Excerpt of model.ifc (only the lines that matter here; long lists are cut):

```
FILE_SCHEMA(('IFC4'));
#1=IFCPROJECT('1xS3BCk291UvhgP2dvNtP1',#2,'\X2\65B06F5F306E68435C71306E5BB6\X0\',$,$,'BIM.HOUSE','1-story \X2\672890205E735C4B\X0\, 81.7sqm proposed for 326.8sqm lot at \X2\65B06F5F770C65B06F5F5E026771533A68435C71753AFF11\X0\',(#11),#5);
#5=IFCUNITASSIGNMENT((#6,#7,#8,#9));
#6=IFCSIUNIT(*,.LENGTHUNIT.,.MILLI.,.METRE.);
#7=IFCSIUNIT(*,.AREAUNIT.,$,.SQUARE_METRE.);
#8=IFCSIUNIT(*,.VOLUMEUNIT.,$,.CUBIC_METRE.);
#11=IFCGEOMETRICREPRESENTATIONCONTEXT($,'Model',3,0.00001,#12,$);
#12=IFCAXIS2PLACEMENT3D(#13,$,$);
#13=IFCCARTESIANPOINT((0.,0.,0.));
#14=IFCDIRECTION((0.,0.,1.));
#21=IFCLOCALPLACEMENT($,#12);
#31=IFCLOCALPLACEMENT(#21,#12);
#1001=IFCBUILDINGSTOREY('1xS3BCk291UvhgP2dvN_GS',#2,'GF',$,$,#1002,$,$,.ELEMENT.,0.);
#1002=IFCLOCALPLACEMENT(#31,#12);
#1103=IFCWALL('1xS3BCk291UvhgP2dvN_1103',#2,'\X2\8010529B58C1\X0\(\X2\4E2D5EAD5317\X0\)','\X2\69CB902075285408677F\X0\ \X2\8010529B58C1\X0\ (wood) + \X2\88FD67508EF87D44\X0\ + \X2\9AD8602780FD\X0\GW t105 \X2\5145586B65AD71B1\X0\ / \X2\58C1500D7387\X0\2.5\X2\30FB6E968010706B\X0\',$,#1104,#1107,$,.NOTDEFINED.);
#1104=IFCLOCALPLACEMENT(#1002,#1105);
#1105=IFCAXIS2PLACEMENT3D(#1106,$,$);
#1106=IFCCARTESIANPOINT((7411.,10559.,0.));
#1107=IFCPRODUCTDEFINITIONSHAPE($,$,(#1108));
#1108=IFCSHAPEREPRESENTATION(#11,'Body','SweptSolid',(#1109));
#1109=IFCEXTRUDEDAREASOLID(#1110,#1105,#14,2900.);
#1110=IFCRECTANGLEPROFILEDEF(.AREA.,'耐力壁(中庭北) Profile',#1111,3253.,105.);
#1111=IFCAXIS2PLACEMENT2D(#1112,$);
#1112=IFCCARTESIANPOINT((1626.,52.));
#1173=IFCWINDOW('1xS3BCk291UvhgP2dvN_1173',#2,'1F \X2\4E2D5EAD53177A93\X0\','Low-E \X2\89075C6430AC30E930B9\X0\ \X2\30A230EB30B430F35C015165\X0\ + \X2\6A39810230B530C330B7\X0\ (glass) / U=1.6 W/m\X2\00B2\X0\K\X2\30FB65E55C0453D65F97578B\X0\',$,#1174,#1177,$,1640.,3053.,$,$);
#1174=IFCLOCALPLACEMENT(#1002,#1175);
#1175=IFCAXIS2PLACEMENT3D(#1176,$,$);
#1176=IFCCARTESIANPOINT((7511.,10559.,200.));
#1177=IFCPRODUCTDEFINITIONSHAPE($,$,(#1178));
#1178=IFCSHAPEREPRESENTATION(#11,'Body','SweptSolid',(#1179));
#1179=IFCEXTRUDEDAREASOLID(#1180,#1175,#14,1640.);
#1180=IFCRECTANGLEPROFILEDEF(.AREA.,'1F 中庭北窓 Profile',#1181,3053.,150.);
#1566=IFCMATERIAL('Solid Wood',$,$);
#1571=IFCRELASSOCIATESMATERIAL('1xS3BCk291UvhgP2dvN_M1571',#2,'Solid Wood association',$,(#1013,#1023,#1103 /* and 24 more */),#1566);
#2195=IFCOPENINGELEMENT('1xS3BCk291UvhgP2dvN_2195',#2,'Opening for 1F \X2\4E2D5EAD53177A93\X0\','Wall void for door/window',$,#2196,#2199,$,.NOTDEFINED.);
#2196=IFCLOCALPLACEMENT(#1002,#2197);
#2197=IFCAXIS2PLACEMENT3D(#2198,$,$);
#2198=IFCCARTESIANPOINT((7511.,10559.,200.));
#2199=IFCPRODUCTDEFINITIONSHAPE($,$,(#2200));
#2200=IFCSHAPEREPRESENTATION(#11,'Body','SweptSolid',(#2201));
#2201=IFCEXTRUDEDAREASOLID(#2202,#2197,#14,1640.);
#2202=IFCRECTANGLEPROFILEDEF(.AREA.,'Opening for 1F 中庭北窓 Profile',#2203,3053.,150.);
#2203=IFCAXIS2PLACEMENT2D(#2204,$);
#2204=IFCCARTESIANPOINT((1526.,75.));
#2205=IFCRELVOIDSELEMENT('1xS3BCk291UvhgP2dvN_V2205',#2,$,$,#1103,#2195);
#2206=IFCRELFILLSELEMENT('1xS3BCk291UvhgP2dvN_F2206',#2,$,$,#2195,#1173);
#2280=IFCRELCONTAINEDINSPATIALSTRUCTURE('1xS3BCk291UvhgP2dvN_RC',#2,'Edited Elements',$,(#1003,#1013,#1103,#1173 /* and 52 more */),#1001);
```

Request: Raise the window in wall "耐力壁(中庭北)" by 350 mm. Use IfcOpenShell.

```python
import numpy as np
import ifcopenshell
import ifcopenshell.api.geometry
import ifcopenshell.util.placement
import ifcopenshell.util.unit

model = ifcopenshell.open("model.ifc")
unit_scale = ifcopenshell.util.unit.calculate_unit_scale(model)

window = model.by_guid("1xS3BCk291UvhgP2dvN_1173")
opening = window.FillsVoids[0].RelatingOpeningElement
dz = 0.35 / unit_scale

shift = np.array([0.0, 0.0, dz])
# The window is not placed relative to its opening, so move both.
for product in (opening, window):
    matrix = ifcopenshell.util.placement.get_local_placement(product.ObjectPlacement)
    matrix[:3, 3] += shift
    ifcopenshell.api.geometry.edit_object_placement(model, product=product, matrix=matrix, is_si=False)

print(f"moved by {dz * unit_scale:+.3f} m")

model.write("model_v2.ifc")
```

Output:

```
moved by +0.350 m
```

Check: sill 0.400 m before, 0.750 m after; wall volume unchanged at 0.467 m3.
